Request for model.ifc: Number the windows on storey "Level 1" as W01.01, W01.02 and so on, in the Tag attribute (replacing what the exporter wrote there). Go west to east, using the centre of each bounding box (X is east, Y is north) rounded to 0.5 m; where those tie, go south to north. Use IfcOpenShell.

First a look at what the model holds.

```python
import ifcopenshell
import ifcopenshell.util.element
import ifcopenshell.util.placement

model = ifcopenshell.open("model.ifc")
print(model.schema)
storey = next(s for s in model.by_type("IfcBuildingStorey") if s.Name == "Level 1")
windows = [e for e in ifcopenshell.util.element.get_decomposition(storey) if e.is_a("IfcWindow")]
for e in sorted(windows, key=lambda e: e.id()):
    origin = ifcopenshell.util.placement.get_local_placement(e.ObjectPlacement)[:3, 3]
    print(e.id(), e.Tag, e.Name, origin.round(2) + 0.0, sep=" | ")
```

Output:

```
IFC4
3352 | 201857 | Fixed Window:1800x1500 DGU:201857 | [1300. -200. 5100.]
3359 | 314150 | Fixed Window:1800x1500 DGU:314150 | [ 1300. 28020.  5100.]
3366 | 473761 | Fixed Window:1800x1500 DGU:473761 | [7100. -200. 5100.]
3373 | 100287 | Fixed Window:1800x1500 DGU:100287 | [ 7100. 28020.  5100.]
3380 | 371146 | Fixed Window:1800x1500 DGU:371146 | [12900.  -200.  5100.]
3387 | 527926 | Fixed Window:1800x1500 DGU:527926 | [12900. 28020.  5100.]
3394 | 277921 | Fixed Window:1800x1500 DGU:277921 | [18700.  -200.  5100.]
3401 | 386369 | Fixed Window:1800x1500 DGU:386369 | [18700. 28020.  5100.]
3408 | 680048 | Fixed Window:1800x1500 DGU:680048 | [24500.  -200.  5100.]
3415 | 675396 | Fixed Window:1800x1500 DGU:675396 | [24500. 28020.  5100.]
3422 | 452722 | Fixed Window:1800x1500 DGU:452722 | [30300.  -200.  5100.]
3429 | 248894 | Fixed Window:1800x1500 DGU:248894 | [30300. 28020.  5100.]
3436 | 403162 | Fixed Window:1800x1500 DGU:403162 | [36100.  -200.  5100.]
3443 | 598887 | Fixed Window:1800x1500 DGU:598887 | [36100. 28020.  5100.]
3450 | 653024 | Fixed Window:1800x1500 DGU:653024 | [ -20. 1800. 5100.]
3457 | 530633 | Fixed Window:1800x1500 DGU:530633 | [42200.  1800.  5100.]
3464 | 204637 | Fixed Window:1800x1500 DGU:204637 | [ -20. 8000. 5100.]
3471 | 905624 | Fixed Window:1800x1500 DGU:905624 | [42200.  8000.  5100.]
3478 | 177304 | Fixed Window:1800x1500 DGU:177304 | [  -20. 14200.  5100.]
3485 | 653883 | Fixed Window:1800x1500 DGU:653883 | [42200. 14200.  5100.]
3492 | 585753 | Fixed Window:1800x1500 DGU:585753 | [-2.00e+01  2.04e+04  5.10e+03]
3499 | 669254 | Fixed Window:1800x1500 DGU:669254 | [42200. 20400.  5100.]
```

```python
import ifcopenshell
import ifcopenshell.geom
import ifcopenshell.util.element
import ifcopenshell.util.shape

model = ifcopenshell.open("model.ifc")
settings = ifcopenshell.geom.settings()
settings.set("use-world-coords", True)


def centre(element):
    shape = ifcopenshell.geom.create_shape(settings, element)
    return ifcopenshell.util.shape.get_bbox_centroid(shape.geometry)


storey = next(s for s in model.by_type("IfcBuildingStorey") if s.Name == "Level 1")
windows = [e for e in ifcopenshell.util.element.get_decomposition(storey) if e.is_a("IfcWindow")]

# Insertion points can sit at a corner or the storey origin, so sort by the geometry (in metres).
centres = {e: centre(e) for e in windows}
windows.sort(key=lambda e: (round(centres[e][0] / 0.5), centres[e][1]))

for i, e in enumerate(windows, start=1):
    number = f"W01.{i:02d}"
    e.Tag = number
    print(e.id(), number)

model.write("model_updated.ifc")
```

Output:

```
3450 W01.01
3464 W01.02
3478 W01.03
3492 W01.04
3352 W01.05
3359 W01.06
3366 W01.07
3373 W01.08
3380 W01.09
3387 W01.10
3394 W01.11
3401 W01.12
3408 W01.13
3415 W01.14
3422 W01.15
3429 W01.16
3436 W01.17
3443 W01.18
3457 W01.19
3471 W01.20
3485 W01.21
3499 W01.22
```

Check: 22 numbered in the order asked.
